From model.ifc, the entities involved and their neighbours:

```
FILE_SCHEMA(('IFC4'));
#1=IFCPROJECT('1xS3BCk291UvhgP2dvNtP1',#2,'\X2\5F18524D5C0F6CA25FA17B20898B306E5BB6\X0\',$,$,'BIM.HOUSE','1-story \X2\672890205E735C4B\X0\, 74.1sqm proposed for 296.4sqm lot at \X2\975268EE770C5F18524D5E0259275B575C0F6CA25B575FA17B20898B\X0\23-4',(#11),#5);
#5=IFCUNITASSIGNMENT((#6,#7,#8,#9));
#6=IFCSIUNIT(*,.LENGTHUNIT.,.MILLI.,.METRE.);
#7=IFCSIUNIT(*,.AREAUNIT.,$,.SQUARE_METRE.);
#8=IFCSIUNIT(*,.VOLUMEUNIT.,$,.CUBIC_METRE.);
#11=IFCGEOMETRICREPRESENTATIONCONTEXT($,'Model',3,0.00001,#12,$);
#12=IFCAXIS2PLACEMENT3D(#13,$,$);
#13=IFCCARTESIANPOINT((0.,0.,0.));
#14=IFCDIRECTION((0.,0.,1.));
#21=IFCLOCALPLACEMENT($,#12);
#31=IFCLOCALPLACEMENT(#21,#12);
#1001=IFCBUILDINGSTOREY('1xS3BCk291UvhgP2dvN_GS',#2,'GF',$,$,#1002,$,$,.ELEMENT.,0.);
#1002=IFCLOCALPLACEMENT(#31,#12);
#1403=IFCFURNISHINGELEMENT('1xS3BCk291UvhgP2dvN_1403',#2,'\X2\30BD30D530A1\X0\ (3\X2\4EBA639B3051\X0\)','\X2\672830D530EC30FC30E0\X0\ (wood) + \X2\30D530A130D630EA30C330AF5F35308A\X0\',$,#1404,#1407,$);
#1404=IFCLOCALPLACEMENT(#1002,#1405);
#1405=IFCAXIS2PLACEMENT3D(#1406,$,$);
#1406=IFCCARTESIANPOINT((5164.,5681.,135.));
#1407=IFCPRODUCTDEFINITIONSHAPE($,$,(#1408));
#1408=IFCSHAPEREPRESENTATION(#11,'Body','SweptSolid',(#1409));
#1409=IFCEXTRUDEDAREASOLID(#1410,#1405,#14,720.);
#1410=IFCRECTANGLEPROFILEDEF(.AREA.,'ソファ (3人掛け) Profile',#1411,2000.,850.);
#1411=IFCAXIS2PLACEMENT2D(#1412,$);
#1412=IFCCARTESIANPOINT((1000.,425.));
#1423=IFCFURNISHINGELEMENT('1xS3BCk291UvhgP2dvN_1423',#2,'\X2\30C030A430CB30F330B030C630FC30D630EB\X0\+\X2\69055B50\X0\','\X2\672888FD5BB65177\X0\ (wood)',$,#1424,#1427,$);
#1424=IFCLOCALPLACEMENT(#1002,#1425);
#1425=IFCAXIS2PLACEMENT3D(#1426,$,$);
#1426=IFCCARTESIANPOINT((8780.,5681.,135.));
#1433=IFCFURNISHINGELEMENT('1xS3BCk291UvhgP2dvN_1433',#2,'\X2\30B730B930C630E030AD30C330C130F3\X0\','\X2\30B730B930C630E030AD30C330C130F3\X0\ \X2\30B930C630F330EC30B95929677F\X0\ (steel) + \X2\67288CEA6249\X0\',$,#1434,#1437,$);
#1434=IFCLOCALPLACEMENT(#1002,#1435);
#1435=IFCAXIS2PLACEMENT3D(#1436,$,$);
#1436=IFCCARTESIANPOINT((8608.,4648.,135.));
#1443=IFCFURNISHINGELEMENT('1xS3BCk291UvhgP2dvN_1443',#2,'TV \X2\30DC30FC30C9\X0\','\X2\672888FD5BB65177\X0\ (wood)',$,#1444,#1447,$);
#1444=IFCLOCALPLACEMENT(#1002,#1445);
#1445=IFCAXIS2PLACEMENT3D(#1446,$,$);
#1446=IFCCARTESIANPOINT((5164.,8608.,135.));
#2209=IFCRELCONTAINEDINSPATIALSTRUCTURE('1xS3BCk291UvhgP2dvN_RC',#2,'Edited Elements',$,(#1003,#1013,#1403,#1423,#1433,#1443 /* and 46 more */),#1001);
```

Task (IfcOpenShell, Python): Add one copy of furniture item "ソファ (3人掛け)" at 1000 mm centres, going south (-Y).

```python
import numpy as np
import ifcopenshell
import ifcopenshell.api.geometry
import ifcopenshell.api.root
import ifcopenshell.util.element
import ifcopenshell.util.placement
import ifcopenshell.util.unit

model = ifcopenshell.open("model.ifc")
unit_scale = ifcopenshell.util.unit.calculate_unit_scale(model)


def reuse_history(source, copy):
    """copy_class also copies each property set's owner history, people and application; keep the originals."""
    for rel in copy.IsDefinedBy:
        if rel.is_a("IfcRelDefinesByProperties") and (history := rel.RelatingPropertyDefinition.OwnerHistory):
            rel.RelatingPropertyDefinition.OwnerHistory = source.OwnerHistory
            ifcopenshell.util.element.remove_deep2(model, history)


source = model.by_id(1403)
base = ifcopenshell.util.placement.get_local_placement(source.ObjectPlacement)
step = np.array([0.0, -1.0, 0.0]) * 1 / unit_scale

for i in range(1, 2):
    copy = ifcopenshell.api.root.copy_class(model, product=source)
    copy.Representation = ifcopenshell.util.element.copy_deep(
        model, source.Representation, exclude=["IfcGeometricRepresentationContext", "IfcRepresentationMap"]
    )
    reuse_history(source, copy)
    matrix = base.copy()
    matrix[:3, 3] += i * step
    print("added at", matrix[:3, 3].round(3) + 0.0)
    ifcopenshell.api.geometry.edit_object_placement(model, product=copy, matrix=matrix, is_si=False)

model.write("model_edited.ifc")
```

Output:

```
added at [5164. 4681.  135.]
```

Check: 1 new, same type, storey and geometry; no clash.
